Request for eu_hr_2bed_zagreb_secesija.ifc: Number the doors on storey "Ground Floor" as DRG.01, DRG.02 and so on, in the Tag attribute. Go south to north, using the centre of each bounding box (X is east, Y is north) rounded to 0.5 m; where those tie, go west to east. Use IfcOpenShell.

First a look at what the model holds.

```python
import ifcopenshell
import ifcopenshell.util.element
import ifcopenshell.util.placement

model = ifcopenshell.open("eu_hr_2bed_zagreb_secesija.ifc")
print(model.schema)
storey = next(s for s in model.by_type("IfcBuildingStorey") if s.Name == "Ground Floor")
doors = [e for e in ifcopenshell.util.element.get_decomposition(storey) if e.is_a("IfcDoor")]
for e in sorted(doors, key=lambda e: e.id()):
    origin = ifcopenshell.util.placement.get_local_placement(e.ObjectPlacement)[:3, 3]
    print(e.id(), e.Tag, e.Name, origin.round(2) + 0.0, sep=" | ")
```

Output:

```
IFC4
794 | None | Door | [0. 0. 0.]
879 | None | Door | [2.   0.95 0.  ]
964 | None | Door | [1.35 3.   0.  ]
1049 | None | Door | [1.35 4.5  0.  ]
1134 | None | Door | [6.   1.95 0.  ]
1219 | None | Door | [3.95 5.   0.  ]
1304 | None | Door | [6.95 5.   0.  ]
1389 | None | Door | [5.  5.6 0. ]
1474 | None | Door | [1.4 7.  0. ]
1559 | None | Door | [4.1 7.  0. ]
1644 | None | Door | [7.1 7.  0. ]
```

```python
import ifcopenshell
import ifcopenshell.geom
import ifcopenshell.util.element
import ifcopenshell.util.shape

model = ifcopenshell.open("eu_hr_2bed_zagreb_secesija.ifc")
settings = ifcopenshell.geom.settings()
settings.set("use-world-coords", True)


def centre(element):
    shape = ifcopenshell.geom.create_shape(settings, element)
    return ifcopenshell.util.shape.get_bbox_centroid(shape.geometry)


storey = next(s for s in model.by_type("IfcBuildingStorey") if s.Name == "Ground Floor")
doors = [e for e in ifcopenshell.util.element.get_decomposition(storey) if e.is_a("IfcDoor")]

# Insertion points can sit at a corner or the storey origin, so sort by the geometry (in metres).
centres = {e: centre(e) for e in doors}
doors.sort(key=lambda e: (round(centres[e][1] / 0.5), centres[e][0]))

for i, e in enumerate(doors, start=1):
    number = f"DRG.{i:02d}"
    e.Tag = number
    print(e.id(), number)

model.write("eu_hr_2bed_zagreb_secesija_v2.ifc")
```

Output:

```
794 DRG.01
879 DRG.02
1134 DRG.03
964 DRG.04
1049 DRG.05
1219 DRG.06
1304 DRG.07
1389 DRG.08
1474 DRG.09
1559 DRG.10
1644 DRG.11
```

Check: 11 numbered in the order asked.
